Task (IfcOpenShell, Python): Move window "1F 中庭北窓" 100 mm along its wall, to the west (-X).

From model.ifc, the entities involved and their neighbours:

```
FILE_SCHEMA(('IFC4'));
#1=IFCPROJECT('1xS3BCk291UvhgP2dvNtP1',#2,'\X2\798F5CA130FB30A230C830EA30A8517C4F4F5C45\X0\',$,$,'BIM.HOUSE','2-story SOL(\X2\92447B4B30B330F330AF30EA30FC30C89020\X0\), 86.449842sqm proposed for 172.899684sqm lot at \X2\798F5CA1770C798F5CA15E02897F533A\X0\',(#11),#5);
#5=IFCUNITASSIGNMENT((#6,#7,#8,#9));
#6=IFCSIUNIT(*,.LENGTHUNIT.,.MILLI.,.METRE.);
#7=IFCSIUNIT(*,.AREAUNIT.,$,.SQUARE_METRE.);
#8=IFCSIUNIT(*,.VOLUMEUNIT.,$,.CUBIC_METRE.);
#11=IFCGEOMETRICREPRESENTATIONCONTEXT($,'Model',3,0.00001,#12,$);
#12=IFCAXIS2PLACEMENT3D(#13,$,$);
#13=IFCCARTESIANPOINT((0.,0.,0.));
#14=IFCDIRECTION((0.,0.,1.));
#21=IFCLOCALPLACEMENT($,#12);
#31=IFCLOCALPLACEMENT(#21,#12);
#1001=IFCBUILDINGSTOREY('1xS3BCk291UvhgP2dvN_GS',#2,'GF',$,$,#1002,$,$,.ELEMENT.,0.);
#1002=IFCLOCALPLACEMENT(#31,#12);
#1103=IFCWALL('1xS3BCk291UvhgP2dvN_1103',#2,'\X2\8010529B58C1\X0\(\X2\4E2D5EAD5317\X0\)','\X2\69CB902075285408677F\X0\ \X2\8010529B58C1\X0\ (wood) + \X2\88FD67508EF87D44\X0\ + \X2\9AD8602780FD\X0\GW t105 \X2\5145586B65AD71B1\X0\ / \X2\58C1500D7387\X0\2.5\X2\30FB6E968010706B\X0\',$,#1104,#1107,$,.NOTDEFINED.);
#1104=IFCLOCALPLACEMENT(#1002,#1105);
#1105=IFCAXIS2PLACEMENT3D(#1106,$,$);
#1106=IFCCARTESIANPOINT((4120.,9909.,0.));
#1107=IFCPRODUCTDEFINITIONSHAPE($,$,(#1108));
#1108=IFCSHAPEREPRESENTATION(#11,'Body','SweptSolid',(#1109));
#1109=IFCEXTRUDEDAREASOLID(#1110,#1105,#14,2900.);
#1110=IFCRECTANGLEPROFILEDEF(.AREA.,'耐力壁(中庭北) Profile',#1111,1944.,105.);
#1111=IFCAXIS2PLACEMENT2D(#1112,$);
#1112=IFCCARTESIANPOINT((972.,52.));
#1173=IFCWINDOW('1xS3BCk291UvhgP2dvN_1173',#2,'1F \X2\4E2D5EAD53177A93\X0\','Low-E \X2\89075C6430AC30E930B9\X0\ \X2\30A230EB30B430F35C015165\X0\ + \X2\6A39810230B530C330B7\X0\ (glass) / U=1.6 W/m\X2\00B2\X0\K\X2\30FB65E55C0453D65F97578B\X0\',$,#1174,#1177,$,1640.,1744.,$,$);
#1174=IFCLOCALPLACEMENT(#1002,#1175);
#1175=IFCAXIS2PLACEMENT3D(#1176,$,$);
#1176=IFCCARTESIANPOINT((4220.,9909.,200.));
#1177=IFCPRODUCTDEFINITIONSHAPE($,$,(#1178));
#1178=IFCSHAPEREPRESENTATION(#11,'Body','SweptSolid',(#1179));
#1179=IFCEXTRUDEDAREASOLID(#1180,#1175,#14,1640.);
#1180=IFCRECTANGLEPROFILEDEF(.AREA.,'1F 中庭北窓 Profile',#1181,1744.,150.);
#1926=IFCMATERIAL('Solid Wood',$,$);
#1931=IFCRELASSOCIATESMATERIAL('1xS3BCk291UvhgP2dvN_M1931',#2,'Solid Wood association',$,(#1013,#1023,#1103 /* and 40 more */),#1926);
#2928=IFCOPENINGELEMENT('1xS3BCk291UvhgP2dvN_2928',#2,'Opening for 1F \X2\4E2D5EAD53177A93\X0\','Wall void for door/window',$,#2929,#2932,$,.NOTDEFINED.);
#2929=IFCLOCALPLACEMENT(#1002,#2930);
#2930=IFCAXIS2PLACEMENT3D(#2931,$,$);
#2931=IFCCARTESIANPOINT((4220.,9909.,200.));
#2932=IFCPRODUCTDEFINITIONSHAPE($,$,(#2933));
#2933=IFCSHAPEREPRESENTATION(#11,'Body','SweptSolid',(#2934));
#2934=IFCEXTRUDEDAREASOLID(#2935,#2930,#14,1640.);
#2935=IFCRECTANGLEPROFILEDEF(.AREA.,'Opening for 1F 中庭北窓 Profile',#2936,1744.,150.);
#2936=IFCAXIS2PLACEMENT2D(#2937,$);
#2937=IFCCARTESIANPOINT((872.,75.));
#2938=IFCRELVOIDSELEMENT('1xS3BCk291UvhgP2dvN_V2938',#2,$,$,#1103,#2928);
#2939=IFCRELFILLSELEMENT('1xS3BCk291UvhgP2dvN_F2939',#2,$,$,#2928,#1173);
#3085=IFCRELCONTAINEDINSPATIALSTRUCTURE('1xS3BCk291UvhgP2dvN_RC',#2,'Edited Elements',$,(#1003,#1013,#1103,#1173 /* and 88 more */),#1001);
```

```python
import ifcopenshell
import ifcopenshell.api.geometry
import ifcopenshell.util.placement
import ifcopenshell.util.unit

model = ifcopenshell.open("model.ifc")
unit_scale = ifcopenshell.util.unit.calculate_unit_scale(model)

window = model.by_guid("1xS3BCk291UvhgP2dvN_1173")
opening = window.FillsVoids[0].RelatingOpeningElement
wall = opening.VoidsElements[0].RelatingBuildingElement

wall_matrix = ifcopenshell.util.placement.get_local_placement(wall.ObjectPlacement)
shift = wall_matrix[:3, 0] * -0.1 / unit_scale
before = ifcopenshell.util.placement.get_local_placement(window.ObjectPlacement)[:3, 3].copy()

# The window is not placed relative to its opening, so move both.
for product in (opening, window):
    matrix = ifcopenshell.util.placement.get_local_placement(product.ObjectPlacement)
    matrix[:3, 3] += shift
    ifcopenshell.api.geometry.edit_object_placement(model, product=product, matrix=matrix, is_si=False)

after = ifcopenshell.util.placement.get_local_placement(window.ObjectPlacement)[:3, 3]
print("window moved by", (after - before).round(3) + 0.0)

model.write("model_edited.ifc")
```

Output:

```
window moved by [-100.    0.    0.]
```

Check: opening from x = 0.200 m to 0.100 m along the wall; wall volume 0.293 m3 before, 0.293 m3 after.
